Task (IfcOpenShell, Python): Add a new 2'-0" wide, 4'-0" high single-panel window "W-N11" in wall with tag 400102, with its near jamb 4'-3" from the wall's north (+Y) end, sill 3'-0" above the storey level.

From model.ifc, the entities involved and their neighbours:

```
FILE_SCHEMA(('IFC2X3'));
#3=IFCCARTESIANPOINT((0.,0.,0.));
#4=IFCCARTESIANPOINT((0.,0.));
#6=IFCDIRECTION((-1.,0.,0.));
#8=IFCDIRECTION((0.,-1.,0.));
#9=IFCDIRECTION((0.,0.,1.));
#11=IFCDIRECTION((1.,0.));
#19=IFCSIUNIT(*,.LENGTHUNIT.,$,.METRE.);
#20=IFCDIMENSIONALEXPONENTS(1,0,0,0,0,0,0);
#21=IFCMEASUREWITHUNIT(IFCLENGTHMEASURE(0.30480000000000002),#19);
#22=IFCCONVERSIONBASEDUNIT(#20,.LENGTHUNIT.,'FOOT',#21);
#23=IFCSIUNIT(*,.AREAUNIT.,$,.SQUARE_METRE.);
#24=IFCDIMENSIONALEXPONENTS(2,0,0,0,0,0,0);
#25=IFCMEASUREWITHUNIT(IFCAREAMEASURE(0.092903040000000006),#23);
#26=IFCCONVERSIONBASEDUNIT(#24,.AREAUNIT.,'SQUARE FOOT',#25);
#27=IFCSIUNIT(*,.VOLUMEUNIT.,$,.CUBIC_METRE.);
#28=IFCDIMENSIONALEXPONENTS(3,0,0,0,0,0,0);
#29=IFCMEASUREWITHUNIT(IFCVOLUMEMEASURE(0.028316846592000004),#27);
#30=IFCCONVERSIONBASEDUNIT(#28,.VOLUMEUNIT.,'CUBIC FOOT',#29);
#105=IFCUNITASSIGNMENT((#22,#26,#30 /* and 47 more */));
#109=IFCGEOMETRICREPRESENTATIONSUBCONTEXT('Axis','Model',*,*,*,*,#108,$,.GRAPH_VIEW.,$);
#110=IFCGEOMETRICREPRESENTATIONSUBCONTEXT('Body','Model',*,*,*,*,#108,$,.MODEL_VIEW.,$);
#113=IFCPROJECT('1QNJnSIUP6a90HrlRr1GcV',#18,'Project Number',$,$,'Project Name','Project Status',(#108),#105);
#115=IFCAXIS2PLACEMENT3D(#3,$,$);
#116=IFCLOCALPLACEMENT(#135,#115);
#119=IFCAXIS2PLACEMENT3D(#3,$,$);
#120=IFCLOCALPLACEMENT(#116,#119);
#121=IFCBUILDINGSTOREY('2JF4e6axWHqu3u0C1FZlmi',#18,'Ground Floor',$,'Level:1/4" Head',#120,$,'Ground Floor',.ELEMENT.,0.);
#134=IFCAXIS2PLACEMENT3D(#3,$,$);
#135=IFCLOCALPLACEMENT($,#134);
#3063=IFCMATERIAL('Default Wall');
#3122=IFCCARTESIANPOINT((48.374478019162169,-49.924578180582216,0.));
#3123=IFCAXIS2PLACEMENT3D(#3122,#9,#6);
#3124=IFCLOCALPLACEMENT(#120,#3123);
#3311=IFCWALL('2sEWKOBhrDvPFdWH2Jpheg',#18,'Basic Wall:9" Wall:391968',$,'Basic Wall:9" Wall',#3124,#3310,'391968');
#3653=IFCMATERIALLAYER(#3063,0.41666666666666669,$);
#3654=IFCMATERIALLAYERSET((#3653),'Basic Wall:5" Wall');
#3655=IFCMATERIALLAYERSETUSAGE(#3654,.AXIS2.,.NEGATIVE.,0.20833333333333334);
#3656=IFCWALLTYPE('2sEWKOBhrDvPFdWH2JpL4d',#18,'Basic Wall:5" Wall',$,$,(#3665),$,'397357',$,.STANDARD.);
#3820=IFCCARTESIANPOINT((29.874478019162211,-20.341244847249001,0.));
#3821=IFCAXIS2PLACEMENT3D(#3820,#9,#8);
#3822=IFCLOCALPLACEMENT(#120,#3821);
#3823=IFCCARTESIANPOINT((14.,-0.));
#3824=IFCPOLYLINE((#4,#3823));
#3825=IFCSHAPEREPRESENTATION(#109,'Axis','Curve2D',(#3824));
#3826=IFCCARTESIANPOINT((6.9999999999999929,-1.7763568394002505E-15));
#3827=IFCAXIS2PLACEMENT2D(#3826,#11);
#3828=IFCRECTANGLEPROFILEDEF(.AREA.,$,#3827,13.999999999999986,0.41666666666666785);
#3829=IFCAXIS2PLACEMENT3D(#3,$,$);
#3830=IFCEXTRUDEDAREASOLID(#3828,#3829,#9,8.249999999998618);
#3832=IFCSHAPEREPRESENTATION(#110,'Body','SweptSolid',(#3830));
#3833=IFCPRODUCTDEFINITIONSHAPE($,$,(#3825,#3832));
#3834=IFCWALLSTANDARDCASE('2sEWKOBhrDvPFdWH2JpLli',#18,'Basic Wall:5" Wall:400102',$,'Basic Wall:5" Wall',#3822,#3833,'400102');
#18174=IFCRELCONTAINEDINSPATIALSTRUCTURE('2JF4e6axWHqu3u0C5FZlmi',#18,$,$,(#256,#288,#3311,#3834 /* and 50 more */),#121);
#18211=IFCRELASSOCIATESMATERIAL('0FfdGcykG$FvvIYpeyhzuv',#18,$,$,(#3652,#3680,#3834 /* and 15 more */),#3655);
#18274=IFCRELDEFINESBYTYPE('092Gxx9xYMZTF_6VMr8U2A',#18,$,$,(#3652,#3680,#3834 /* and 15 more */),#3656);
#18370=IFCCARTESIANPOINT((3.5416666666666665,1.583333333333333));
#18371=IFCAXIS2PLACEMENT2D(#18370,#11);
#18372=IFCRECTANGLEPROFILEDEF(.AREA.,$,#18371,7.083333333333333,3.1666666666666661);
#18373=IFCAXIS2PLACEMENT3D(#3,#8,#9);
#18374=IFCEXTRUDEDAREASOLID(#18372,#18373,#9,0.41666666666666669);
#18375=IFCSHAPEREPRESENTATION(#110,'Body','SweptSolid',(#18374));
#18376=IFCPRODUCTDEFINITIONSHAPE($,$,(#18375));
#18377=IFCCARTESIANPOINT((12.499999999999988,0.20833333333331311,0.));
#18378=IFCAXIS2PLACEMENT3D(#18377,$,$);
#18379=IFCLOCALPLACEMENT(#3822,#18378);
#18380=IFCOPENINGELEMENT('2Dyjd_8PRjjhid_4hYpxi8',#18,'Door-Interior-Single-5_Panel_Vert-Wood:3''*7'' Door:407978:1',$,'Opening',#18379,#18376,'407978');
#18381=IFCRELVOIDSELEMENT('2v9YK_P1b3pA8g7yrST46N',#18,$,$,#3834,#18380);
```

```python
import numpy as np
import ifcopenshell
import ifcopenshell.api.feature
import ifcopenshell.api.geometry
import ifcopenshell.api.root
import ifcopenshell.api.spatial
import ifcopenshell.api.type
import ifcopenshell.geom
import ifcopenshell.util.element
import ifcopenshell.util.placement
import ifcopenshell.util.representation
import ifcopenshell.util.shape
import ifcopenshell.util.unit

model = ifcopenshell.open("model.ifc")
unit_scale = ifcopenshell.util.unit.calculate_unit_scale(model)
settings = ifcopenshell.geom.settings()


def volume(element):
    """Net volume in cubic metres, openings subtracted."""
    shape = ifcopenshell.geom.create_shape(settings, element)
    return ifcopenshell.util.shape.get_volume(shape.geometry)


wall = model.by_id(3834)
storey = ifcopenshell.util.element.get_container(wall, ifc_class="IfcBuildingStorey")
context = ifcopenshell.util.representation.get_context(model, "Model", "Body", "MODEL_VIEW")
before = volume(wall)

width, height, from_end, sill = 0.6096, 1.2192, 1.2954, 0.9144  # metres

# The wall runs along its own X axis, and the end named is its -X end.
wall_shape = ifcopenshell.geom.create_shape(settings, wall)
x, y, z = ifcopenshell.util.shape.get_vertices(wall_shape.geometry).T
start = x.min() + from_end
face, thickness = float(y.min()), float(y.max() - y.min())
wall_matrix = ifcopenshell.util.placement.get_local_placement(wall.ObjectPlacement)
level = ifcopenshell.util.placement.get_local_placement(storey.ObjectPlacement)[2, 3]


def in_wall(x, y):
    """Placement at x, y metres in the wall's axes, at sill height."""
    matrix = wall_matrix.copy()
    matrix[:, 3] = wall_matrix @ np.array([x / unit_scale, y / unit_scale, 0.0, 1.0])
    matrix[2, 3] = level + sill / unit_scale
    return matrix


# Opening: a box that overshoots both wall faces by 50 mm.
opening = ifcopenshell.api.root.create_entity(model, ifc_class="IfcOpeningElement")
box = ifcopenshell.api.geometry.add_wall_representation(
    model, context=context, length=width, height=height, thickness=thickness + 0.1
)
ifcopenshell.api.geometry.assign_representation(model, product=opening, representation=box)
ifcopenshell.api.geometry.edit_object_placement(model, product=opening, matrix=in_wall(start, face - 0.05), is_si=False)
ifcopenshell.api.feature.add_feature(model, feature=opening, element=wall)

window = ifcopenshell.api.root.create_entity(model, ifc_class="IfcWindow", name="W-N11")
window.OverallWidth, window.OverallHeight = width / unit_scale, height / unit_scale
body = ifcopenshell.api.geometry.add_window_representation(
    model,
    context=context,
    overall_width=window.OverallWidth,
    overall_height=window.OverallHeight,
    partition_type="SINGLE_PANEL",
)
ifcopenshell.api.geometry.assign_representation(model, product=window, representation=body)
ifcopenshell.api.spatial.assign_container(model, products=[window], relating_structure=storey)
fills = ifcopenshell.api.feature.add_filling(model, opening=opening, element=window)
fills.OwnerHistory = window.OwnerHistory  # required in IFC2X3

# IFC2X3 keeps the operation on the window style.
style = ifcopenshell.api.root.create_entity(model, ifc_class="IfcWindowStyle", name="W-N11")
style.OperationType, style.ConstructionType = "SINGLE_PANEL", "NOTDEFINED"
style.ParameterTakesPrecedence = style.Sizeable = False
ifcopenshell.api.type.assign_type(model, related_objects=[window], relating_type=style)

# Centre the window in the wall's thickness.
ifcopenshell.api.geometry.edit_object_placement(model, product=window, matrix=in_wall(start, face), is_si=False)
window_shape = ifcopenshell.geom.create_shape(settings, window)
depth = ifcopenshell.util.shape.get_vertices(window_shape.geometry)[:, 1]
offset = face + thickness / 2 - (depth.min() + depth.max()) / 2
ifcopenshell.api.geometry.edit_object_placement(model, product=window, matrix=in_wall(start, offset), is_si=False)

after = volume(wall)

print(f"wall volume {before:.3f} -> {after:.3f} m3")

model.write("model_v2.ifc")
```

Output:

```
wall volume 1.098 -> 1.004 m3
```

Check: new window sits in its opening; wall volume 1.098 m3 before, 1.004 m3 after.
